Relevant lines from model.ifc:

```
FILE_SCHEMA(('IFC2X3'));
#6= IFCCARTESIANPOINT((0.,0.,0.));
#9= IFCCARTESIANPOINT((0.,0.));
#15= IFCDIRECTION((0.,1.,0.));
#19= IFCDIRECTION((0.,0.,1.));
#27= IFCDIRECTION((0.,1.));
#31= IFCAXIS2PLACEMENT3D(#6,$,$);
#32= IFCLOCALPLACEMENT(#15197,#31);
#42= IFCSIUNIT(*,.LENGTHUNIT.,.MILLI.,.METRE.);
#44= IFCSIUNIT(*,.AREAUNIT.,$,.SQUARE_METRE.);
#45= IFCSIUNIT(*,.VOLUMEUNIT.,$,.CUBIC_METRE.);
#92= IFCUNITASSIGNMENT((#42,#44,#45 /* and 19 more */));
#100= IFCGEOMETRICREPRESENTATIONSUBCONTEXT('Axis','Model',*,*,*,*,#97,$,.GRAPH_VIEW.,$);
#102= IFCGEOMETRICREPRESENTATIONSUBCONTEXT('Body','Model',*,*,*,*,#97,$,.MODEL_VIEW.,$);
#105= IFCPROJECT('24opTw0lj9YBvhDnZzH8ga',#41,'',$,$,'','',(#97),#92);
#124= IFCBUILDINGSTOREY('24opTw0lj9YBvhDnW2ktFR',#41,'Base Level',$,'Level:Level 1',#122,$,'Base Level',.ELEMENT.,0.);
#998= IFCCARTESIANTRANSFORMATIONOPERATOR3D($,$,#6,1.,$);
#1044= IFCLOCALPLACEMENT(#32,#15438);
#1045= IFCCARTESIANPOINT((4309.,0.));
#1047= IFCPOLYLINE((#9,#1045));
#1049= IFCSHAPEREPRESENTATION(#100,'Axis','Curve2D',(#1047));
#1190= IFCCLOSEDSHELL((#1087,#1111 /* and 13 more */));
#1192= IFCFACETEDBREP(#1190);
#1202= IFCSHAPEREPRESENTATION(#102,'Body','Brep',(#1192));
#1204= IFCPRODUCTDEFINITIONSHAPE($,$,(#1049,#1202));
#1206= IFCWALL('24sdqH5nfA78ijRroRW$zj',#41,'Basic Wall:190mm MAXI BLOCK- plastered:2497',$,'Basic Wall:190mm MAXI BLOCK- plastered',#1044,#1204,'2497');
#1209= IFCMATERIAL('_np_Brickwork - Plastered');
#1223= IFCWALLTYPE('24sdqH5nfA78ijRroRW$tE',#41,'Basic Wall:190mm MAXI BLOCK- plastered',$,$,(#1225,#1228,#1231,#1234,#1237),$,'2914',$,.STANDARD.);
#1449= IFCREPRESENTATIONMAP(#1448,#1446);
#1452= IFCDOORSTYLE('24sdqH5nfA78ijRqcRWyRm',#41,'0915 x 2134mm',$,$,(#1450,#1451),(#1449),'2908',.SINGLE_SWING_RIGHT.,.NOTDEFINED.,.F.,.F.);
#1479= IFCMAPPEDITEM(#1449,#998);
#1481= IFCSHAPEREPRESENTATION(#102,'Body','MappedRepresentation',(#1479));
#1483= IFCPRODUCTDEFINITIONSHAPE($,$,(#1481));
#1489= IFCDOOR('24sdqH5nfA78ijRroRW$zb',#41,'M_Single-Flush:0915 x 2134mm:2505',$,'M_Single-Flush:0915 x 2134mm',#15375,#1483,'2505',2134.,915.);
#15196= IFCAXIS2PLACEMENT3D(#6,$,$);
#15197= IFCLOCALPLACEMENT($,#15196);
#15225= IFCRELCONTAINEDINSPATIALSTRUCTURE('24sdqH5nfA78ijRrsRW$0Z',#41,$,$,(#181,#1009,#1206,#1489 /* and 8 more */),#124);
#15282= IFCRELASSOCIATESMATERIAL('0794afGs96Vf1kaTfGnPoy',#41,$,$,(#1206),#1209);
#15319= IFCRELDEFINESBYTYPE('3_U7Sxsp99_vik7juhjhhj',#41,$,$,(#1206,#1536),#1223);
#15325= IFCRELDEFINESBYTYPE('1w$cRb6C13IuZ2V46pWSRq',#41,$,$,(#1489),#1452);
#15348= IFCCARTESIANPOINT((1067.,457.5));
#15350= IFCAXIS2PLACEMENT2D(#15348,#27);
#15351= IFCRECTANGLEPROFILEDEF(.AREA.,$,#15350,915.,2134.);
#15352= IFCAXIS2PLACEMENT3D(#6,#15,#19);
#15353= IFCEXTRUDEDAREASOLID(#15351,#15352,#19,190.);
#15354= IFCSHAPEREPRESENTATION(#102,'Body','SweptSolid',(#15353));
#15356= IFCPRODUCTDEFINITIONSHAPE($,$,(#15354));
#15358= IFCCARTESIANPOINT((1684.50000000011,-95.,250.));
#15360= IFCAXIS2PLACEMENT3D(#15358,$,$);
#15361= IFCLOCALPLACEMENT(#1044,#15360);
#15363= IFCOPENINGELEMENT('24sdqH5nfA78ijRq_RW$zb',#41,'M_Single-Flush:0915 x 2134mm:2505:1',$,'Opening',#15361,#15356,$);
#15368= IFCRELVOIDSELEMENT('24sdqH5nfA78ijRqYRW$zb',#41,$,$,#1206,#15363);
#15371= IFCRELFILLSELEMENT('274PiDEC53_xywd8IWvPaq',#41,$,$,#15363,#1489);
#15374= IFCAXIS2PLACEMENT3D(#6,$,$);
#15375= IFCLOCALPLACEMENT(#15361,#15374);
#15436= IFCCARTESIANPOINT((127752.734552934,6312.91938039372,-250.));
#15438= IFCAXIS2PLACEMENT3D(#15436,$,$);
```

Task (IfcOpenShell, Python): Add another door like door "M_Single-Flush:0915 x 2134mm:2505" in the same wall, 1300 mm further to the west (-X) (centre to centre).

```python
import ifcopenshell
import ifcopenshell.api.feature
import ifcopenshell.api.geometry
import ifcopenshell.api.root
import ifcopenshell.geom
import ifcopenshell.util.element
import ifcopenshell.util.placement
import ifcopenshell.util.shape
import ifcopenshell.util.unit

model = ifcopenshell.open("model.ifc")
unit_scale = ifcopenshell.util.unit.calculate_unit_scale(model)
settings = ifcopenshell.geom.settings()


def volume(element):
    """Net volume in cubic metres, openings subtracted."""
    shape = ifcopenshell.geom.create_shape(settings, element)
    return ifcopenshell.util.shape.get_volume(shape.geometry)


def reuse_history(source, copy):
    """copy_class also copies each property set's owner history, people and application; keep the originals."""
    for rel in copy.IsDefinedBy:
        if rel.is_a("IfcRelDefinesByProperties") and (history := rel.RelatingPropertyDefinition.OwnerHistory):
            rel.RelatingPropertyDefinition.OwnerHistory = source.OwnerHistory
            ifcopenshell.util.element.remove_deep2(model, history)


door = model.by_guid("24sdqH5nfA78ijRroRW$zb")
opening = door.FillsVoids[0].RelatingOpeningElement
wall = opening.VoidsElements[0].RelatingBuildingElement
before = volume(wall)
shift = ifcopenshell.util.placement.get_local_placement(wall.ObjectPlacement)[:3, 0] * -1.3 / unit_scale

# copy_class copies the void relationship, type, container and properties, but no geometry.
new_opening = ifcopenshell.api.root.copy_class(model, product=opening)
new_opening.Representation = ifcopenshell.util.element.copy_deep(
    model, opening.Representation, exclude=["IfcGeometricRepresentationContext", "IfcRepresentationMap"]
)
new_opening.Name = "M_Single-Flush:0915 x 2134mm"
new_door = ifcopenshell.api.root.copy_class(model, product=door)
new_door.Representation = ifcopenshell.util.element.copy_deep(
    model, door.Representation, exclude=["IfcGeometricRepresentationContext", "IfcRepresentationMap"]
)
new_door.Name = "M_Single-Flush:0915 x 2134mm"
new_door.Tag = None
reuse_history(door, new_door)
fills = ifcopenshell.api.feature.add_filling(model, opening=new_opening, element=new_door)
fills.OwnerHistory = new_door.OwnerHistory  # required in IFC2X3

for old, new in ((opening, new_opening), (door, new_door)):
    matrix = ifcopenshell.util.placement.get_local_placement(old.ObjectPlacement)
    matrix[:3, 3] += shift
    ifcopenshell.api.geometry.edit_object_placement(model, product=new, matrix=matrix, is_si=False)

after = volume(wall)

print(f"wall volume {before:.3f} -> {after:.3f} m3")

model.write("model_edited.ifc")
```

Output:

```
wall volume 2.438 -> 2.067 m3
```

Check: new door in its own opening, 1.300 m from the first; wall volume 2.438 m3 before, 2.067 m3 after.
